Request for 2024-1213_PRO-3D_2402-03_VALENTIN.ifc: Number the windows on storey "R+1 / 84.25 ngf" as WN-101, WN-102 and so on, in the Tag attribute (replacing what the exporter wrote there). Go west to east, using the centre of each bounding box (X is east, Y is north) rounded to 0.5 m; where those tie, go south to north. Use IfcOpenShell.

First a look at what the model holds.

```python
import ifcopenshell
import ifcopenshell.util.element
import ifcopenshell.util.placement

model = ifcopenshell.open("2024-1213_PRO-3D_2402-03_VALENTIN.ifc")
print(model.schema)
storey = next(s for s in model.by_type("IfcBuildingStorey") if s.Name == "R+1 / 84.25 ngf")
windows = [e for e in ifcopenshell.util.element.get_decomposition(storey) if e.is_a("IfcWindow")]
for e in sorted(windows, key=lambda e: e.id()):
    origin = ifcopenshell.util.placement.get_local_placement(e.ObjectPlacement)[:3, 3]
    print(e.id(), e.Tag, e.Name, origin.round(2) + 0.0, sep=" | ")
```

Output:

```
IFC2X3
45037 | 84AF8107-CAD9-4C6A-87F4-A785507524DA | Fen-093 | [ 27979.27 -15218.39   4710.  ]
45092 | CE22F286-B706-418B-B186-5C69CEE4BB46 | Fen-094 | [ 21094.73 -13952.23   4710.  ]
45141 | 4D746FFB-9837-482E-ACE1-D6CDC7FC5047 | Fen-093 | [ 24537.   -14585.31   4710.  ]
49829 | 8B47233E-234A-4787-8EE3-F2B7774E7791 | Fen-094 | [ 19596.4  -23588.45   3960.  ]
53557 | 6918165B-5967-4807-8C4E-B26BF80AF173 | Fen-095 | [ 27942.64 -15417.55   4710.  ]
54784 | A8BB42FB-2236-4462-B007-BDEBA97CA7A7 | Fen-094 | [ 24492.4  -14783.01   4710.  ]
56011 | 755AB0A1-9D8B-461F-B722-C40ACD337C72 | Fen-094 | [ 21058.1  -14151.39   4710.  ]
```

```python
import ifcopenshell
import ifcopenshell.geom
import ifcopenshell.util.element
import ifcopenshell.util.shape

model = ifcopenshell.open("2024-1213_PRO-3D_2402-03_VALENTIN.ifc")
settings = ifcopenshell.geom.settings()
settings.set("use-world-coords", True)


def centre(element):
    shape = ifcopenshell.geom.create_shape(settings, element)
    return ifcopenshell.util.shape.get_bbox_centroid(shape.geometry)


storey = next(s for s in model.by_type("IfcBuildingStorey") if s.Name == "R+1 / 84.25 ngf")
windows = [e for e in ifcopenshell.util.element.get_decomposition(storey) if e.is_a("IfcWindow")]

# Insertion points can sit at a corner or the storey origin, so sort by the geometry (in metres).
centres = {e: centre(e) for e in windows}
windows.sort(key=lambda e: (round(centres[e][0] / 0.5), centres[e][1]))

for i, e in enumerate(windows, start=1):
    number = f"WN-1{i:02d}"
    e.Tag = number
    print(e.id(), number)

model.write("2024-1213_PRO-3D_2402-03_VALENTIN_rev.ifc")
```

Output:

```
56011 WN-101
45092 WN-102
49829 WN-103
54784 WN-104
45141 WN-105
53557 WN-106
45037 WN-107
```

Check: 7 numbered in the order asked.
